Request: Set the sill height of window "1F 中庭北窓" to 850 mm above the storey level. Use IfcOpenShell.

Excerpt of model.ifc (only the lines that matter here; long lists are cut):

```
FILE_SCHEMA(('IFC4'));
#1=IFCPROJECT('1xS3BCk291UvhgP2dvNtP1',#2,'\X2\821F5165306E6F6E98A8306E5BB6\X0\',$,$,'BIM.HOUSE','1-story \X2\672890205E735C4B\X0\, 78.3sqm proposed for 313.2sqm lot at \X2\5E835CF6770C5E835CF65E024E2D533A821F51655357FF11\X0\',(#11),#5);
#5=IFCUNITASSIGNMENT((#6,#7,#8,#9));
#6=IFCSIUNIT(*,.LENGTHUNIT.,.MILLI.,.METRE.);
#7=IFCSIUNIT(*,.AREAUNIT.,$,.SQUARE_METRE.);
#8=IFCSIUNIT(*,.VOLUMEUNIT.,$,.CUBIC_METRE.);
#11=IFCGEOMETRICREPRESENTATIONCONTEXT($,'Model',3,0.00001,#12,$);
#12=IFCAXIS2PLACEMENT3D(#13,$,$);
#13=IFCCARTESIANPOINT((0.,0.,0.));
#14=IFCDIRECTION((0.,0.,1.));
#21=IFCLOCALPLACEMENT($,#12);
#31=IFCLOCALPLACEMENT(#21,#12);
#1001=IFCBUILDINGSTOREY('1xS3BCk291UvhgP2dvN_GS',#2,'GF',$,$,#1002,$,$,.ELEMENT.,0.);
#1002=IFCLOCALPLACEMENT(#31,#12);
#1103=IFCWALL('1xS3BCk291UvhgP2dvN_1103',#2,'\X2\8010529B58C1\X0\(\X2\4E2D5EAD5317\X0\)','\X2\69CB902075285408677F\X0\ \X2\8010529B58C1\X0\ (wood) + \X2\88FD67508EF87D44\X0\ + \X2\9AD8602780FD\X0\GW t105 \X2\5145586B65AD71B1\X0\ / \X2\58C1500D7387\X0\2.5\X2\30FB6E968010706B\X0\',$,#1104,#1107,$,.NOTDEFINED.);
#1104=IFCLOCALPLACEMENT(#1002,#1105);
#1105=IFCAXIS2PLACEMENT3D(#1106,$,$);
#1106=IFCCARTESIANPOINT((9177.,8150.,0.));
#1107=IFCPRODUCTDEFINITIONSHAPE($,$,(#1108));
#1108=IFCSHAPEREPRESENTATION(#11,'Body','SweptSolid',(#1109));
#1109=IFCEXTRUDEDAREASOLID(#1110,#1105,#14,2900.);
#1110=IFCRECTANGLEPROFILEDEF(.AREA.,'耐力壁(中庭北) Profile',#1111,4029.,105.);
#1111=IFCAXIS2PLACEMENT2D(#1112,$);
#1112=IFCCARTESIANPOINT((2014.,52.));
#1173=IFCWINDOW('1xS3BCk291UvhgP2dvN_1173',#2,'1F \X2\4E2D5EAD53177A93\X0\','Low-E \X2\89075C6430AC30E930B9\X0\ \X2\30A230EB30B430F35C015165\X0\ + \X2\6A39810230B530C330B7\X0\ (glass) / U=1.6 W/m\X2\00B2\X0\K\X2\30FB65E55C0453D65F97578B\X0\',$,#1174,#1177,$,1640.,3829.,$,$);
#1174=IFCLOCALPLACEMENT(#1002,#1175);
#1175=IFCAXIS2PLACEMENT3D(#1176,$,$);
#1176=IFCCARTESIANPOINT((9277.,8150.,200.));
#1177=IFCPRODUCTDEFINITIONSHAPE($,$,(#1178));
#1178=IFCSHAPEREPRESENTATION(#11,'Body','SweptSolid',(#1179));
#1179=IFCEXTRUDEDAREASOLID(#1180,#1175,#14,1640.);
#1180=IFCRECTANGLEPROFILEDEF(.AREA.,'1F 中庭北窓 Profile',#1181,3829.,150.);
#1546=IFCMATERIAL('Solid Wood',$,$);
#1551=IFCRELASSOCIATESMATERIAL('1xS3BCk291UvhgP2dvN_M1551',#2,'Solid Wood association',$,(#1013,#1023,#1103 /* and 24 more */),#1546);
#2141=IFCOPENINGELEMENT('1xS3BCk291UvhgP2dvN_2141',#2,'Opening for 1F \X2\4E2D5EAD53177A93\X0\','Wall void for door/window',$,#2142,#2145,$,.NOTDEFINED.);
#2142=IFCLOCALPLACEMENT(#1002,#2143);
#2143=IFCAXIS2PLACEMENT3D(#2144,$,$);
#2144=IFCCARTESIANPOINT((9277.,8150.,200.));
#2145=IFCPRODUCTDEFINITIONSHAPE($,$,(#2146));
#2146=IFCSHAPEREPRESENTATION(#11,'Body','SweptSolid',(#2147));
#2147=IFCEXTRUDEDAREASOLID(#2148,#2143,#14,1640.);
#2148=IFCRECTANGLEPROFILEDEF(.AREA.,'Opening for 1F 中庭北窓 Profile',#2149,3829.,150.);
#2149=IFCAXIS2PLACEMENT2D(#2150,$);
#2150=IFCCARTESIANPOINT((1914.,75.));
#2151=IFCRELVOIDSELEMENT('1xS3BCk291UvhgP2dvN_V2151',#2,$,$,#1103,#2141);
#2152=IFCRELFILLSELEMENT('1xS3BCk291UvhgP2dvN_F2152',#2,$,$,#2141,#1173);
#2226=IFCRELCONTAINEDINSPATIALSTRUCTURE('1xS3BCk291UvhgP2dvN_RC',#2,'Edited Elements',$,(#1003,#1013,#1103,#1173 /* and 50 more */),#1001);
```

```python
import numpy as np
import ifcopenshell
import ifcopenshell.api.geometry
import ifcopenshell.geom
import ifcopenshell.util.element
import ifcopenshell.util.placement
import ifcopenshell.util.shape
import ifcopenshell.util.unit

model = ifcopenshell.open("model.ifc")
unit_scale = ifcopenshell.util.unit.calculate_unit_scale(model)

window = model.by_guid("1xS3BCk291UvhgP2dvN_1173")
opening = window.FillsVoids[0].RelatingOpeningElement
storey = ifcopenshell.util.element.get_container(window, ifc_class="IfcBuildingStorey")
level = ifcopenshell.util.placement.get_local_placement(storey.ObjectPlacement)[2, 3]

# The opening's origin need not be at the sill, so measure its lowest point.
shape = ifcopenshell.geom.create_shape(ifcopenshell.geom.settings(), opening)
bottom = ifcopenshell.util.shape.get_shape_bottom_elevation(shape, shape.geometry) / unit_scale
dz = level + 0.85 / unit_scale - bottom

shift = np.array([0.0, 0.0, dz])
# The window is not placed relative to its opening, so move both.
for product in (opening, window):
    matrix = ifcopenshell.util.placement.get_local_placement(product.ObjectPlacement)
    matrix[:3, 3] += shift
    ifcopenshell.api.geometry.edit_object_placement(model, product=product, matrix=matrix, is_si=False)

print(f"moved by {dz * unit_scale:+.3f} m")

model.write("model_v2.ifc")
```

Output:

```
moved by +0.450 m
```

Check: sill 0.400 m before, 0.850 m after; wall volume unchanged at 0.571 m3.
